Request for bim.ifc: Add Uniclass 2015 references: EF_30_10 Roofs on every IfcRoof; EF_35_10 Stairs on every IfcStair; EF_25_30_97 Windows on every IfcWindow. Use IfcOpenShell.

First a look at what the model holds.

```python
import ifcopenshell

model = ifcopenshell.open("bim.ifc")
print(model.schema)
print("classifications:", [c.Name for c in model.by_type("IfcClassification")])
for ifc_class in ("IfcDoor", "IfcRoof", "IfcStair", "IfcWall", "IfcWindow"):
    print(ifc_class, len(model.by_type(ifc_class)))
```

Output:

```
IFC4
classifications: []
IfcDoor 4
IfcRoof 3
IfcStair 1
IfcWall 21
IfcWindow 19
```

```python
import ifcopenshell
import ifcopenshell.api.classification

model = ifcopenshell.open("bim.ifc")

system = ifcopenshell.api.classification.add_classification(model, classification="Uniclass 2015")

codes = {
    "IfcRoof": ("EF_30_10", "Roofs"),
    "IfcStair": ("EF_35_10", "Stairs"),
    "IfcWindow": ("EF_25_30_97", "Windows"),
}
for ifc_class, (code, name) in codes.items():
    products = model.by_type(ifc_class)
    ifcopenshell.api.classification.add_reference(
        model, products=products, classification=system, identification=code, name=name
    )
    print(code, len(products))

model.write("bim_rev.ifc")
```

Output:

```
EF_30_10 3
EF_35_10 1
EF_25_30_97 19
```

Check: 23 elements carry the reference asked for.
